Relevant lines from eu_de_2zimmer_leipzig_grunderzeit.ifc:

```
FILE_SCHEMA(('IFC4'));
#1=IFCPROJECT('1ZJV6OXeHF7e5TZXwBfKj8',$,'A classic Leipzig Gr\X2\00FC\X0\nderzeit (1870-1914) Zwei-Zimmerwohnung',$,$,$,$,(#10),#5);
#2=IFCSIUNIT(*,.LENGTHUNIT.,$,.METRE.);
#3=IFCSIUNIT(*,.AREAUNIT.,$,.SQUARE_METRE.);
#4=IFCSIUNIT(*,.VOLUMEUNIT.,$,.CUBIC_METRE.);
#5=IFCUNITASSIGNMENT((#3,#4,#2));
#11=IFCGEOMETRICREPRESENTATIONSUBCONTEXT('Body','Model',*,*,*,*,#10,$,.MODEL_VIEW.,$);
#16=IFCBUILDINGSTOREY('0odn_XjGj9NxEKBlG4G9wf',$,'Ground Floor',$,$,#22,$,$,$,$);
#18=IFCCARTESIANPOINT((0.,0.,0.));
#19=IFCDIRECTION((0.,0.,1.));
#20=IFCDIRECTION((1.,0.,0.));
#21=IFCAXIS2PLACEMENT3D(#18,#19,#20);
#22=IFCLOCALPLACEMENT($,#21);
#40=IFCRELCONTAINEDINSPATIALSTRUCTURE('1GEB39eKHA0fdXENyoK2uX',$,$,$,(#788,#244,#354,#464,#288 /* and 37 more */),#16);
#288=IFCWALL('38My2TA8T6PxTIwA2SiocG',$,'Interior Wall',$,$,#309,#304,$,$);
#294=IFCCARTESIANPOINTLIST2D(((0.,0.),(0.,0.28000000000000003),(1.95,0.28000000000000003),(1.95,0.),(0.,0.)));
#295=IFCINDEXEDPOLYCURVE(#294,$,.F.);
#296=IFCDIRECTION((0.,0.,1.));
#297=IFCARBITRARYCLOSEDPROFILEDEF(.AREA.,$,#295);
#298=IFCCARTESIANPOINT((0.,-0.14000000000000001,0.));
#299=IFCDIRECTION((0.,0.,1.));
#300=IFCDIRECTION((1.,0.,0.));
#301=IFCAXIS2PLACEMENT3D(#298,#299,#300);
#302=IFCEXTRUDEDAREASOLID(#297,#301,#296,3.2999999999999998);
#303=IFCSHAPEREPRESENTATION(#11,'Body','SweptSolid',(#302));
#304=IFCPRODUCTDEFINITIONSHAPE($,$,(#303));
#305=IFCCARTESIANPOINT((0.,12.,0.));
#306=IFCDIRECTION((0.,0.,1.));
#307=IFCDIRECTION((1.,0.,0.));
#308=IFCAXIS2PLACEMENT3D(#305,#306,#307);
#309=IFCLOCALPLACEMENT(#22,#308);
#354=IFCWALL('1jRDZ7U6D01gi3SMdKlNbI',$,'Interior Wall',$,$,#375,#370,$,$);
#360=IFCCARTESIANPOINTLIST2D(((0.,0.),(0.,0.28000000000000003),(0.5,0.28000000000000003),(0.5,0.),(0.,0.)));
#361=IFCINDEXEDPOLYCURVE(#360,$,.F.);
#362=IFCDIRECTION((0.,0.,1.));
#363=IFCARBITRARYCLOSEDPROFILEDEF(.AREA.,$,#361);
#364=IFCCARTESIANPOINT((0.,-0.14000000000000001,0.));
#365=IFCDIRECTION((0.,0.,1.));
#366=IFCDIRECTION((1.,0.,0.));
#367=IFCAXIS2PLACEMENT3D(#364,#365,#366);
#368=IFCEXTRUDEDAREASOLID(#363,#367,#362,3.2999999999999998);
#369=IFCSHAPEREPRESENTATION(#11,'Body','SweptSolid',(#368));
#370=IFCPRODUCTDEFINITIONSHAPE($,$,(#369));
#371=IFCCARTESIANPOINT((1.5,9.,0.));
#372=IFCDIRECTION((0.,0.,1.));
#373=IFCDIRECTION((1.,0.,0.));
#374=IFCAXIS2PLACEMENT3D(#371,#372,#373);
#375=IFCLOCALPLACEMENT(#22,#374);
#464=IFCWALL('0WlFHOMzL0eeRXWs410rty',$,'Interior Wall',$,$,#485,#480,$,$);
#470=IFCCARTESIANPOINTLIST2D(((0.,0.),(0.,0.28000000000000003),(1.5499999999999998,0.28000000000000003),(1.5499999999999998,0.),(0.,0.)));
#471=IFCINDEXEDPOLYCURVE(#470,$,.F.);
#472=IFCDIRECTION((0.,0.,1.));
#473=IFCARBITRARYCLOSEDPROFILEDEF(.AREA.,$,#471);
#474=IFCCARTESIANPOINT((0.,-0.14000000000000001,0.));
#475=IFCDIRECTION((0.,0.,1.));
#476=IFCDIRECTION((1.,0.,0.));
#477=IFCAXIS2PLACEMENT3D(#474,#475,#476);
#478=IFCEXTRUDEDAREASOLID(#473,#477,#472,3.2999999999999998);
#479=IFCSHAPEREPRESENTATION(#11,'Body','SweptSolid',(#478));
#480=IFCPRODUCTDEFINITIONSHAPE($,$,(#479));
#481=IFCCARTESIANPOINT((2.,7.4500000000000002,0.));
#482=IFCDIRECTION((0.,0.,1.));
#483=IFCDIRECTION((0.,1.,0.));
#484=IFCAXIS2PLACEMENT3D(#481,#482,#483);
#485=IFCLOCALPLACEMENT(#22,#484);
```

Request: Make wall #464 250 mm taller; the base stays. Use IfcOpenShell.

```python
import ifcopenshell
import ifcopenshell.geom
import ifcopenshell.util.representation
import ifcopenshell.util.shape

model = ifcopenshell.open("eu_de_2zimmer_leipzig_grunderzeit.ifc")
settings = ifcopenshell.geom.settings()


def volume(element):
    """Net volume in cubic metres, openings subtracted."""
    shape = ifcopenshell.geom.create_shape(settings, element)
    return ifcopenshell.util.shape.get_volume(shape.geometry)


wall = model.by_guid("0WlFHOMzL0eeRXWs410rty")
before = volume(wall)

body = ifcopenshell.util.representation.get_representation(wall, "Model", "Body")
solid = body.Items[0]
old_height = solid.Depth
solid.Depth += 0.25
after = volume(wall)

print(f"height {old_height:g} -> {solid.Depth:g}, volume {before:.3f} -> {after:.3f} m3")

model.write("eu_de_2zimmer_leipzig_grunderzeit-out.ifc")
```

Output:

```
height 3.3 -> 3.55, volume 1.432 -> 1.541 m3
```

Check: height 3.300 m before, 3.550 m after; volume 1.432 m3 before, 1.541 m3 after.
